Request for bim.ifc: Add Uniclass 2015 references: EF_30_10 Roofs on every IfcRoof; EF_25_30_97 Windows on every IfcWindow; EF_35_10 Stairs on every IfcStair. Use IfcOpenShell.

First a look at what the model holds.

```python
import ifcopenshell

model = ifcopenshell.open("bim.ifc")
print(model.schema)
print("classifications:", [c.Name for c in model.by_type("IfcClassification")])
for ifc_class in ("IfcDoor", "IfcRoof", "IfcStair", "IfcWall", "IfcWindow"):
    print(ifc_class, len(model.by_type(ifc_class)))
```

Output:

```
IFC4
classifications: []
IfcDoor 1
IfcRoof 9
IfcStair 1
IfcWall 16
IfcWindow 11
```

```python
import ifcopenshell
import ifcopenshell.api.classification

model = ifcopenshell.open("bim.ifc")

system = ifcopenshell.api.classification.add_classification(model, classification="Uniclass 2015")

codes = {
    "IfcRoof": ("EF_30_10", "Roofs"),
    "IfcWindow": ("EF_25_30_97", "Windows"),
    "IfcStair": ("EF_35_10", "Stairs"),
}
for ifc_class, (code, name) in codes.items():
    products = model.by_type(ifc_class)
    ifcopenshell.api.classification.add_reference(
        model, products=products, classification=system, identification=code, name=name
    )
    print(code, len(products))

model.write("bim_updated.ifc")
```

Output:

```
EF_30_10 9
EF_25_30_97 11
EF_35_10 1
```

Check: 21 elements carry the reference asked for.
